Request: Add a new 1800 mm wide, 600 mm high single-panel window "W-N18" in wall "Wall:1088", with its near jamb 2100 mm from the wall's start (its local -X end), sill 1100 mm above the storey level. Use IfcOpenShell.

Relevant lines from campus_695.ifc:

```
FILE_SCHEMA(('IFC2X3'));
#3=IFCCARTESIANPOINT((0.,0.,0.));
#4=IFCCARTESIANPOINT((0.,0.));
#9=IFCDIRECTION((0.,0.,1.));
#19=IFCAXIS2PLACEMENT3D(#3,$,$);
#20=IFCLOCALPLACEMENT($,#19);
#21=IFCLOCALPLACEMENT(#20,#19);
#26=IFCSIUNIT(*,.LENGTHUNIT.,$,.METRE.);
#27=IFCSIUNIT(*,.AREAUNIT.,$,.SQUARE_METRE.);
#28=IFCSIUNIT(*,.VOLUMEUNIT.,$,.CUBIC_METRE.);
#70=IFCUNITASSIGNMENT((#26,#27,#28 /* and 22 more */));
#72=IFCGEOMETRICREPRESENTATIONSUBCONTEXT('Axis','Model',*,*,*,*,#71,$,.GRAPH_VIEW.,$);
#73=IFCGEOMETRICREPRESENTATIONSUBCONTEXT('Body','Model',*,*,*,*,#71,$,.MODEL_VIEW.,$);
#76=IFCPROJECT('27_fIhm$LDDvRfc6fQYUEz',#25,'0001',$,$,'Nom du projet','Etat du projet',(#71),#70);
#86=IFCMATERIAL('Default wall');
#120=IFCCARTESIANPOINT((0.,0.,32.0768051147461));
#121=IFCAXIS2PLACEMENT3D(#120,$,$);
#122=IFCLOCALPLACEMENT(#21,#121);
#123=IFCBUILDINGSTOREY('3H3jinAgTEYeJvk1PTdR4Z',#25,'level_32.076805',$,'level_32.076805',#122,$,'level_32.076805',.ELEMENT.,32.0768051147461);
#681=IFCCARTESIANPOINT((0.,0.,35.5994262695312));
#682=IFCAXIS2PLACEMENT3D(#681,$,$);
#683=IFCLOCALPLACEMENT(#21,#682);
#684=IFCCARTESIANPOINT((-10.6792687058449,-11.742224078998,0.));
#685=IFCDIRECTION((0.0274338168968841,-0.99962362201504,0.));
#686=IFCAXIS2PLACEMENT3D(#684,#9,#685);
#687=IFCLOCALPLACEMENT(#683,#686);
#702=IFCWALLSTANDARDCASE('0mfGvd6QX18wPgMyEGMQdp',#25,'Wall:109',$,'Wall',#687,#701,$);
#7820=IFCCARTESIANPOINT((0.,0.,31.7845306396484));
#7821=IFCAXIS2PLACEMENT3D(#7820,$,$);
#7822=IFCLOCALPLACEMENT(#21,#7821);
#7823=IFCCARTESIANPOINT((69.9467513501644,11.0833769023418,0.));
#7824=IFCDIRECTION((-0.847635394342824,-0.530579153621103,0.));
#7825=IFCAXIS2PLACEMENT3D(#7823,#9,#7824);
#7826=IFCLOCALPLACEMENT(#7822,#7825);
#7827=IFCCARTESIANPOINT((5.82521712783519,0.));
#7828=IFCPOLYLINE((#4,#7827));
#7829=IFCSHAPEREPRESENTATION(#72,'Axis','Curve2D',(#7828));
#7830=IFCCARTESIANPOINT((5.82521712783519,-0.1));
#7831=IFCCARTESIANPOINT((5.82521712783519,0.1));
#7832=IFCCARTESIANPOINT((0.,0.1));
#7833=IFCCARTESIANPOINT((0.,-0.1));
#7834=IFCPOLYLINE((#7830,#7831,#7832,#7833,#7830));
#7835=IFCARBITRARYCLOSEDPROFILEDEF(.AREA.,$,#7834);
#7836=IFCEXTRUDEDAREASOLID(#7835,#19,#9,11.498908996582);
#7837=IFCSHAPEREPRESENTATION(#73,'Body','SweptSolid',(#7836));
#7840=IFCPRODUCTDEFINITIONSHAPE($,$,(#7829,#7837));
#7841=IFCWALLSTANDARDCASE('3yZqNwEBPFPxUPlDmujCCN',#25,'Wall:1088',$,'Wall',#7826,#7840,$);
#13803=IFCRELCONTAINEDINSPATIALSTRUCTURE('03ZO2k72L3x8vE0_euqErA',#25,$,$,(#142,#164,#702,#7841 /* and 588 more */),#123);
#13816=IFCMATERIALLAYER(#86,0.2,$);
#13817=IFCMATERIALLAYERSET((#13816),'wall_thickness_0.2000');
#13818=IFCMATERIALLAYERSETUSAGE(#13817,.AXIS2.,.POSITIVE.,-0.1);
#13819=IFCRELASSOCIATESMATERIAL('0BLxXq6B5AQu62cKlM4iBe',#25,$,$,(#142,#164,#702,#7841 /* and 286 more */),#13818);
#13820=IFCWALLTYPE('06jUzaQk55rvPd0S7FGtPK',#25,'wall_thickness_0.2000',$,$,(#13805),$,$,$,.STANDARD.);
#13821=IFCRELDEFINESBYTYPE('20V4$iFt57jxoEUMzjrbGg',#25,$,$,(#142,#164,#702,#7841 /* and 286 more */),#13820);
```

```python
import numpy as np
import ifcopenshell
import ifcopenshell.api.feature
import ifcopenshell.api.geometry
import ifcopenshell.api.root
import ifcopenshell.api.spatial
import ifcopenshell.api.type
import ifcopenshell.geom
import ifcopenshell.util.element
import ifcopenshell.util.placement
import ifcopenshell.util.representation
import ifcopenshell.util.shape
import ifcopenshell.util.unit

model = ifcopenshell.open("campus_695.ifc")
unit_scale = ifcopenshell.util.unit.calculate_unit_scale(model)
settings = ifcopenshell.geom.settings()


def volume(element):
    """Net volume in cubic metres, openings subtracted."""
    shape = ifcopenshell.geom.create_shape(settings, element)
    return ifcopenshell.util.shape.get_volume(shape.geometry)


wall = model.by_guid("3yZqNwEBPFPxUPlDmujCCN")
storey = ifcopenshell.util.element.get_container(wall, ifc_class="IfcBuildingStorey")
context = ifcopenshell.util.representation.get_context(model, "Model", "Body", "MODEL_VIEW")
before = volume(wall)

width, height, from_end, sill = 1.8, 0.6, 2.1, 1.1  # metres

# The wall runs along its own X axis, and the end named is its -X end.
wall_shape = ifcopenshell.geom.create_shape(settings, wall)
x, y, z = ifcopenshell.util.shape.get_vertices(wall_shape.geometry).T
start = x.min() + from_end
face, thickness = float(y.min()), float(y.max() - y.min())
wall_matrix = ifcopenshell.util.placement.get_local_placement(wall.ObjectPlacement)
level = ifcopenshell.util.placement.get_local_placement(storey.ObjectPlacement)[2, 3]


def in_wall(x, y):
    """Placement at x, y metres in the wall's axes, at sill height."""
    matrix = wall_matrix.copy()
    matrix[:, 3] = wall_matrix @ np.array([x / unit_scale, y / unit_scale, 0.0, 1.0])
    matrix[2, 3] = level + sill / unit_scale
    return matrix


# Opening: a box that overshoots both wall faces by 50 mm.
opening = ifcopenshell.api.root.create_entity(model, ifc_class="IfcOpeningElement")
box = ifcopenshell.api.geometry.add_wall_representation(
    model, context=context, length=width, height=height, thickness=thickness + 0.1
)
ifcopenshell.api.geometry.assign_representation(model, product=opening, representation=box)
ifcopenshell.api.geometry.edit_object_placement(model, product=opening, matrix=in_wall(start, face - 0.05), is_si=False)
ifcopenshell.api.feature.add_feature(model, feature=opening, element=wall)

window = ifcopenshell.api.root.create_entity(model, ifc_class="IfcWindow", name="W-N18")
window.OverallWidth, window.OverallHeight = width / unit_scale, height / unit_scale
body = ifcopenshell.api.geometry.add_window_representation(
    model,
    context=context,
    overall_width=window.OverallWidth,
    overall_height=window.OverallHeight,
    partition_type="SINGLE_PANEL",
)
ifcopenshell.api.geometry.assign_representation(model, product=window, representation=body)
ifcopenshell.api.spatial.assign_container(model, products=[window], relating_structure=storey)
fills = ifcopenshell.api.feature.add_filling(model, opening=opening, element=window)
fills.OwnerHistory = window.OwnerHistory  # required in IFC2X3

# IFC2X3 keeps the operation on the window style.
style = ifcopenshell.api.root.create_entity(model, ifc_class="IfcWindowStyle", name="W-N18")
style.OperationType, style.ConstructionType = "SINGLE_PANEL", "NOTDEFINED"
style.ParameterTakesPrecedence = style.Sizeable = False
ifcopenshell.api.type.assign_type(model, related_objects=[window], relating_type=style)

# Centre the window in the wall's thickness.
ifcopenshell.api.geometry.edit_object_placement(model, product=window, matrix=in_wall(start, face), is_si=False)
window_shape = ifcopenshell.geom.create_shape(settings, window)
depth = ifcopenshell.util.shape.get_vertices(window_shape.geometry)[:, 1]
offset = face + thickness / 2 - (depth.min() + depth.max()) / 2
ifcopenshell.api.geometry.edit_object_placement(model, product=window, matrix=in_wall(start, offset), is_si=False)

after = volume(wall)

print(f"wall volume {before:.3f} -> {after:.3f} m3")

model.write("campus_695_edited.ifc")
```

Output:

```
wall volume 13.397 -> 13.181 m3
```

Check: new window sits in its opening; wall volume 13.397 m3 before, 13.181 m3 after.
